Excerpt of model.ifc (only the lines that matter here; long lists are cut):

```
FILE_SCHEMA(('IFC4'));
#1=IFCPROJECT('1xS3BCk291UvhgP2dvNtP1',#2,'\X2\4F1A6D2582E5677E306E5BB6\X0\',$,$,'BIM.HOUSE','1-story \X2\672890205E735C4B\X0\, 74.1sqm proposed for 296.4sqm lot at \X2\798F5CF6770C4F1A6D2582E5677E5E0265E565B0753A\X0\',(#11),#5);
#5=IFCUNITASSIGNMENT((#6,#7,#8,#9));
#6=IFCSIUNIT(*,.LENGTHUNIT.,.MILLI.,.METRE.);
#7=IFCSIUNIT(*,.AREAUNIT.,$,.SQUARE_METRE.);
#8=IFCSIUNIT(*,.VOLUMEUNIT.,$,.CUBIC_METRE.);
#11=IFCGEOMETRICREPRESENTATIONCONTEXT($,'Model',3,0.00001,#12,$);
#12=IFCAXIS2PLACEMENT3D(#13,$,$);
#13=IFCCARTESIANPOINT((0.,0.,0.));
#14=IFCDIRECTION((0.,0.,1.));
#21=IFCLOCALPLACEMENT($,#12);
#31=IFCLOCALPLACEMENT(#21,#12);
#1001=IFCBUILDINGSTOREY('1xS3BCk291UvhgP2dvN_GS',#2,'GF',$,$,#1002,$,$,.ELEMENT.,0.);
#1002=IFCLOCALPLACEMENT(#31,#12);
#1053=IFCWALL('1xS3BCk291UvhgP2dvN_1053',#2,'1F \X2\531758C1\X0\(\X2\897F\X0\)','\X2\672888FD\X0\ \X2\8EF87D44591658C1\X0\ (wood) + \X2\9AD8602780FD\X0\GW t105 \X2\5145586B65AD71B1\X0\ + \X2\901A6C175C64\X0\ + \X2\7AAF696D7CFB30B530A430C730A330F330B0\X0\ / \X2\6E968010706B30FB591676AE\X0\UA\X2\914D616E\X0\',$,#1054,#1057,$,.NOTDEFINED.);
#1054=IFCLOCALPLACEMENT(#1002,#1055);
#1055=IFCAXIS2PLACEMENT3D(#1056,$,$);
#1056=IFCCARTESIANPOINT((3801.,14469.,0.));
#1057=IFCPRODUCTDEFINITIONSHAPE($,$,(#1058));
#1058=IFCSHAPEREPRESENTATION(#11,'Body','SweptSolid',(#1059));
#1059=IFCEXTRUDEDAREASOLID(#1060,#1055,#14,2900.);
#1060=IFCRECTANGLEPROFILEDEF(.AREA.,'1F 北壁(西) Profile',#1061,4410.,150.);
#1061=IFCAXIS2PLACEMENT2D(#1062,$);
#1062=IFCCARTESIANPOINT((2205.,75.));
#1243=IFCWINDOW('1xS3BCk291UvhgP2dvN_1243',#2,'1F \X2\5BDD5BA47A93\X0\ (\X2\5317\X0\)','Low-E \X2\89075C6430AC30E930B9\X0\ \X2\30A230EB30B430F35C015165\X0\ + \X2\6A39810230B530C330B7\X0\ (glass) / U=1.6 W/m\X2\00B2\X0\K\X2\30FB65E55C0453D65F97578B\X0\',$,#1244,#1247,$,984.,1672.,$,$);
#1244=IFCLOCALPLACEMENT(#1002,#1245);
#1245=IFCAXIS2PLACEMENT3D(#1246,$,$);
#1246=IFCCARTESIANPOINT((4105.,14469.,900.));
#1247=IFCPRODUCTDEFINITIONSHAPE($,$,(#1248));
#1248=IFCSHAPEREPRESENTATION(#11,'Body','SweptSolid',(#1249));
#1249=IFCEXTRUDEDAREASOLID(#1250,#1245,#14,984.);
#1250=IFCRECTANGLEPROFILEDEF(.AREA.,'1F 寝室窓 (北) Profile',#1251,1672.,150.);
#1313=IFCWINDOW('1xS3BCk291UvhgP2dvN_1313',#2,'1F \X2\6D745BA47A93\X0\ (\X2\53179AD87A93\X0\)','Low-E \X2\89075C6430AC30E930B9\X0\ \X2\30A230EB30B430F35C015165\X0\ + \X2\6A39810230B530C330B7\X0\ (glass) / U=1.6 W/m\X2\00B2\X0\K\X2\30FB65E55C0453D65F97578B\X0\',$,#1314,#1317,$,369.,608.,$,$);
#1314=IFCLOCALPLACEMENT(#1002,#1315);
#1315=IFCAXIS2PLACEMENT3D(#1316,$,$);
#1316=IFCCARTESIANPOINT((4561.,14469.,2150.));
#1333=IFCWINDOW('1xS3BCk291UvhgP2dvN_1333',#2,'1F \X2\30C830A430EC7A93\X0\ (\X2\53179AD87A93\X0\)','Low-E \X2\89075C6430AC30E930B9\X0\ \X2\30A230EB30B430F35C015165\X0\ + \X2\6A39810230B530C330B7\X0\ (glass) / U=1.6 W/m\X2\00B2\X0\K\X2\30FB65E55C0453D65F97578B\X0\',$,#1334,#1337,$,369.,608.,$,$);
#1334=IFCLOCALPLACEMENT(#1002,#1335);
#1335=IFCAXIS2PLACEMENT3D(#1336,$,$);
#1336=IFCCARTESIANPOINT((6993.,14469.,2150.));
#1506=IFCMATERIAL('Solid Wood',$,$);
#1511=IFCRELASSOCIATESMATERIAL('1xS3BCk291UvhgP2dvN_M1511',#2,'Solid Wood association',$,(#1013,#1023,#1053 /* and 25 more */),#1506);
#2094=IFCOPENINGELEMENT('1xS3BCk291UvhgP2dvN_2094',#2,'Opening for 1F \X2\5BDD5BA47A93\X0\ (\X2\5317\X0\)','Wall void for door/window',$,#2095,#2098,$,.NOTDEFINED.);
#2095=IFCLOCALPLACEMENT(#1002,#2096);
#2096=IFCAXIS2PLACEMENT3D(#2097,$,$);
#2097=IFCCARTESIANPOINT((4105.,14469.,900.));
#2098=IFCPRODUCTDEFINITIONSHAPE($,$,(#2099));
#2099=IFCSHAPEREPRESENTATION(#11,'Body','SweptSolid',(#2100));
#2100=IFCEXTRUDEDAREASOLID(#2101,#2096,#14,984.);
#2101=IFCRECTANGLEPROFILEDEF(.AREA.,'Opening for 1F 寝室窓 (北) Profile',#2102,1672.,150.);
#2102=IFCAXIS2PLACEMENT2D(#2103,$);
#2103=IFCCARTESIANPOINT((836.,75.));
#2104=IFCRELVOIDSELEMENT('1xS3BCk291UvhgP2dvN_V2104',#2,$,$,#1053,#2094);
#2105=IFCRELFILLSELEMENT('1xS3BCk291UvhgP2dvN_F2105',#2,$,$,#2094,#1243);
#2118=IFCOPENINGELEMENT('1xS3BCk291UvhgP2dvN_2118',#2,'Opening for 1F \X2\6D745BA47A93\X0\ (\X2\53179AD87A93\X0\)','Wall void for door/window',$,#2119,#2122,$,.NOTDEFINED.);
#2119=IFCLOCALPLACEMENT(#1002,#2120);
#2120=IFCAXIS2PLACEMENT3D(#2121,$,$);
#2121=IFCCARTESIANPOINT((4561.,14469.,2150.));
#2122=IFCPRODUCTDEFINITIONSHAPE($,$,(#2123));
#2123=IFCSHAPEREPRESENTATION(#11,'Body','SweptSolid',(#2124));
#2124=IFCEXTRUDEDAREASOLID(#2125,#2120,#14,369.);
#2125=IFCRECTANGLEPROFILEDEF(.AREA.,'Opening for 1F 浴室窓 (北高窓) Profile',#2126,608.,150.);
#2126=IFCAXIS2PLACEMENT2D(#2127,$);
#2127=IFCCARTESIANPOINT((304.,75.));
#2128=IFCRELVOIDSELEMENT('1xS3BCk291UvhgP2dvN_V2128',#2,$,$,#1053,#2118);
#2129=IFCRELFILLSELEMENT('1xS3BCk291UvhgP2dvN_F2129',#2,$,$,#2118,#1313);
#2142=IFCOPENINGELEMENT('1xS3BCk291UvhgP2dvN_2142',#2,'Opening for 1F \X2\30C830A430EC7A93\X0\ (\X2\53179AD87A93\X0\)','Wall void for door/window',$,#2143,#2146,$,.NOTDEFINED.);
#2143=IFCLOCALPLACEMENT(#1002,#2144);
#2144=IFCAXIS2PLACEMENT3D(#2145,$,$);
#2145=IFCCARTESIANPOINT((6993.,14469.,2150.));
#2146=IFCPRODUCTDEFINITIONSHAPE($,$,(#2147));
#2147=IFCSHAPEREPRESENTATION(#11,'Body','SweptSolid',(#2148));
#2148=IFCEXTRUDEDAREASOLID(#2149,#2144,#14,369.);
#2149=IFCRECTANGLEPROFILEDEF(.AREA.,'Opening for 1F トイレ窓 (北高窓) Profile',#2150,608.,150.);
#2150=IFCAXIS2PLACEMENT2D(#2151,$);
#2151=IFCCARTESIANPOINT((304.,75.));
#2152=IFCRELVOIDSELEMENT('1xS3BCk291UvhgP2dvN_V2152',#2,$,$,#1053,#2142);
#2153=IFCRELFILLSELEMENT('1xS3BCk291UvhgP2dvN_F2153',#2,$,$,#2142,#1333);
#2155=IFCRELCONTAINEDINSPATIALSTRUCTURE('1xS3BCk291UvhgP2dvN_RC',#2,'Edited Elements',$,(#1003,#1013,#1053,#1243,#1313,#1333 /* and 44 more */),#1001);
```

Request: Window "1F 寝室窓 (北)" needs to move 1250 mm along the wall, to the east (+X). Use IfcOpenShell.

```python
import ifcopenshell
import ifcopenshell.api.geometry
import ifcopenshell.util.placement

model = ifcopenshell.open("model.ifc")

window = model.by_guid("1xS3BCk291UvhgP2dvN_1243")
opening = window.FillsVoids[0].RelatingOpeningElement
wall = opening.VoidsElements[0].RelatingBuildingElement

wall_matrix = ifcopenshell.util.placement.get_local_placement(wall.ObjectPlacement)
shift = wall_matrix[:3, 0] * 1250.0
before = ifcopenshell.util.placement.get_local_placement(window.ObjectPlacement)[:3, 3].copy()

# The window is not placed relative to its opening, so move both.
for product in (opening, window):
    matrix = ifcopenshell.util.placement.get_local_placement(product.ObjectPlacement)
    matrix[:3, 3] += shift
    ifcopenshell.api.geometry.edit_object_placement(model, product=product, matrix=matrix, is_si=False)

after = ifcopenshell.util.placement.get_local_placement(window.ObjectPlacement)[:3, 3]
print("window moved by", (after - before).round(3) + 0.0)

model.write("model_edited.ifc")
```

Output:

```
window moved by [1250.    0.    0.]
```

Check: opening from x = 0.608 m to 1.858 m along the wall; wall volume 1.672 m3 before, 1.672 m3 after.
